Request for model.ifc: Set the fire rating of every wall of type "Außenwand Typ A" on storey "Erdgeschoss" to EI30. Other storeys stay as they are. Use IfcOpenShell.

First a look at what the model holds.

```python
import ifcopenshell
import ifcopenshell.util.element

model = ifcopenshell.open("model.ifc")
print(model.schema)
storey = next(s for s in model.by_type("IfcBuildingStorey") if s.Name == "Erdgeschoss")
walls = [e for e in ifcopenshell.util.element.get_decomposition(storey) if e.is_a("IfcWall")]
seen = {}
for e in walls:
    element_type = ifcopenshell.util.element.get_type(e)
    key = (element_type.Name if element_type != e and element_type else None, ifcopenshell.util.element.get_pset(e, "Pset_WallCommon", "FireRating"))
    seen[key] = seen.get(key, 0) + 1
for (name, value), count in sorted(seen.items(), key=str):
    print(count, "x", name, "|", value)
```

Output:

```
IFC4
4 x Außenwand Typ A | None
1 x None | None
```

```python
import ifcopenshell
import ifcopenshell.api.pset
import ifcopenshell.util.element

model = ifcopenshell.open("model.ifc")

storey = next(s for s in model.by_type("IfcBuildingStorey") if s.Name == "Erdgeschoss")
walls = [e for e in ifcopenshell.util.element.get_decomposition(storey) if e.is_a("IfcWall")]

count = 0
for e in walls:
    element_type = ifcopenshell.util.element.get_type(e)
    if element_type in (None, e) or element_type.Name != "Außenwand Typ A":
        continue
    # add_pset returns the element's existing set when there is one.
    pset = ifcopenshell.api.pset.add_pset(model, product=e, name="Pset_WallCommon")
    ifcopenshell.api.pset.edit_pset(model, pset=pset, properties={"FireRating": "EI30"})
    count += 1

print(count, "walls updated")

model.write("model_v2.ifc")
```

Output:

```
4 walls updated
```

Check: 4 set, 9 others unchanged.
